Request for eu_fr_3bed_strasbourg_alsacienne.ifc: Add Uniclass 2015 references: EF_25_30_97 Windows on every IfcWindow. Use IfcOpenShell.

First a look at what the model holds.

```python
import ifcopenshell

model = ifcopenshell.open("eu_fr_3bed_strasbourg_alsacienne.ifc")
print(model.schema)
print("classifications:", [c.Name for c in model.by_type("IfcClassification")])
for ifc_class in ("IfcDoor", "IfcRoof", "IfcStair", "IfcWall", "IfcWindow"):
    print(ifc_class, len(model.by_type(ifc_class)))
```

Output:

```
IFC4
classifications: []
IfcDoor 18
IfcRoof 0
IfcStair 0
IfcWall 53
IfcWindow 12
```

```python
import ifcopenshell
import ifcopenshell.api.classification

model = ifcopenshell.open("eu_fr_3bed_strasbourg_alsacienne.ifc")

system = ifcopenshell.api.classification.add_classification(model, classification="Uniclass 2015")

codes = {
    "IfcWindow": ("EF_25_30_97", "Windows"),
}
for ifc_class, (code, name) in codes.items():
    products = model.by_type(ifc_class)
    ifcopenshell.api.classification.add_reference(
        model, products=products, classification=system, identification=code, name=name
    )
    print(code, len(products))

model.write("eu_fr_3bed_strasbourg_alsacienne-out.ifc")
```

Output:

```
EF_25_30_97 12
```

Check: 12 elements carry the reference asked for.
